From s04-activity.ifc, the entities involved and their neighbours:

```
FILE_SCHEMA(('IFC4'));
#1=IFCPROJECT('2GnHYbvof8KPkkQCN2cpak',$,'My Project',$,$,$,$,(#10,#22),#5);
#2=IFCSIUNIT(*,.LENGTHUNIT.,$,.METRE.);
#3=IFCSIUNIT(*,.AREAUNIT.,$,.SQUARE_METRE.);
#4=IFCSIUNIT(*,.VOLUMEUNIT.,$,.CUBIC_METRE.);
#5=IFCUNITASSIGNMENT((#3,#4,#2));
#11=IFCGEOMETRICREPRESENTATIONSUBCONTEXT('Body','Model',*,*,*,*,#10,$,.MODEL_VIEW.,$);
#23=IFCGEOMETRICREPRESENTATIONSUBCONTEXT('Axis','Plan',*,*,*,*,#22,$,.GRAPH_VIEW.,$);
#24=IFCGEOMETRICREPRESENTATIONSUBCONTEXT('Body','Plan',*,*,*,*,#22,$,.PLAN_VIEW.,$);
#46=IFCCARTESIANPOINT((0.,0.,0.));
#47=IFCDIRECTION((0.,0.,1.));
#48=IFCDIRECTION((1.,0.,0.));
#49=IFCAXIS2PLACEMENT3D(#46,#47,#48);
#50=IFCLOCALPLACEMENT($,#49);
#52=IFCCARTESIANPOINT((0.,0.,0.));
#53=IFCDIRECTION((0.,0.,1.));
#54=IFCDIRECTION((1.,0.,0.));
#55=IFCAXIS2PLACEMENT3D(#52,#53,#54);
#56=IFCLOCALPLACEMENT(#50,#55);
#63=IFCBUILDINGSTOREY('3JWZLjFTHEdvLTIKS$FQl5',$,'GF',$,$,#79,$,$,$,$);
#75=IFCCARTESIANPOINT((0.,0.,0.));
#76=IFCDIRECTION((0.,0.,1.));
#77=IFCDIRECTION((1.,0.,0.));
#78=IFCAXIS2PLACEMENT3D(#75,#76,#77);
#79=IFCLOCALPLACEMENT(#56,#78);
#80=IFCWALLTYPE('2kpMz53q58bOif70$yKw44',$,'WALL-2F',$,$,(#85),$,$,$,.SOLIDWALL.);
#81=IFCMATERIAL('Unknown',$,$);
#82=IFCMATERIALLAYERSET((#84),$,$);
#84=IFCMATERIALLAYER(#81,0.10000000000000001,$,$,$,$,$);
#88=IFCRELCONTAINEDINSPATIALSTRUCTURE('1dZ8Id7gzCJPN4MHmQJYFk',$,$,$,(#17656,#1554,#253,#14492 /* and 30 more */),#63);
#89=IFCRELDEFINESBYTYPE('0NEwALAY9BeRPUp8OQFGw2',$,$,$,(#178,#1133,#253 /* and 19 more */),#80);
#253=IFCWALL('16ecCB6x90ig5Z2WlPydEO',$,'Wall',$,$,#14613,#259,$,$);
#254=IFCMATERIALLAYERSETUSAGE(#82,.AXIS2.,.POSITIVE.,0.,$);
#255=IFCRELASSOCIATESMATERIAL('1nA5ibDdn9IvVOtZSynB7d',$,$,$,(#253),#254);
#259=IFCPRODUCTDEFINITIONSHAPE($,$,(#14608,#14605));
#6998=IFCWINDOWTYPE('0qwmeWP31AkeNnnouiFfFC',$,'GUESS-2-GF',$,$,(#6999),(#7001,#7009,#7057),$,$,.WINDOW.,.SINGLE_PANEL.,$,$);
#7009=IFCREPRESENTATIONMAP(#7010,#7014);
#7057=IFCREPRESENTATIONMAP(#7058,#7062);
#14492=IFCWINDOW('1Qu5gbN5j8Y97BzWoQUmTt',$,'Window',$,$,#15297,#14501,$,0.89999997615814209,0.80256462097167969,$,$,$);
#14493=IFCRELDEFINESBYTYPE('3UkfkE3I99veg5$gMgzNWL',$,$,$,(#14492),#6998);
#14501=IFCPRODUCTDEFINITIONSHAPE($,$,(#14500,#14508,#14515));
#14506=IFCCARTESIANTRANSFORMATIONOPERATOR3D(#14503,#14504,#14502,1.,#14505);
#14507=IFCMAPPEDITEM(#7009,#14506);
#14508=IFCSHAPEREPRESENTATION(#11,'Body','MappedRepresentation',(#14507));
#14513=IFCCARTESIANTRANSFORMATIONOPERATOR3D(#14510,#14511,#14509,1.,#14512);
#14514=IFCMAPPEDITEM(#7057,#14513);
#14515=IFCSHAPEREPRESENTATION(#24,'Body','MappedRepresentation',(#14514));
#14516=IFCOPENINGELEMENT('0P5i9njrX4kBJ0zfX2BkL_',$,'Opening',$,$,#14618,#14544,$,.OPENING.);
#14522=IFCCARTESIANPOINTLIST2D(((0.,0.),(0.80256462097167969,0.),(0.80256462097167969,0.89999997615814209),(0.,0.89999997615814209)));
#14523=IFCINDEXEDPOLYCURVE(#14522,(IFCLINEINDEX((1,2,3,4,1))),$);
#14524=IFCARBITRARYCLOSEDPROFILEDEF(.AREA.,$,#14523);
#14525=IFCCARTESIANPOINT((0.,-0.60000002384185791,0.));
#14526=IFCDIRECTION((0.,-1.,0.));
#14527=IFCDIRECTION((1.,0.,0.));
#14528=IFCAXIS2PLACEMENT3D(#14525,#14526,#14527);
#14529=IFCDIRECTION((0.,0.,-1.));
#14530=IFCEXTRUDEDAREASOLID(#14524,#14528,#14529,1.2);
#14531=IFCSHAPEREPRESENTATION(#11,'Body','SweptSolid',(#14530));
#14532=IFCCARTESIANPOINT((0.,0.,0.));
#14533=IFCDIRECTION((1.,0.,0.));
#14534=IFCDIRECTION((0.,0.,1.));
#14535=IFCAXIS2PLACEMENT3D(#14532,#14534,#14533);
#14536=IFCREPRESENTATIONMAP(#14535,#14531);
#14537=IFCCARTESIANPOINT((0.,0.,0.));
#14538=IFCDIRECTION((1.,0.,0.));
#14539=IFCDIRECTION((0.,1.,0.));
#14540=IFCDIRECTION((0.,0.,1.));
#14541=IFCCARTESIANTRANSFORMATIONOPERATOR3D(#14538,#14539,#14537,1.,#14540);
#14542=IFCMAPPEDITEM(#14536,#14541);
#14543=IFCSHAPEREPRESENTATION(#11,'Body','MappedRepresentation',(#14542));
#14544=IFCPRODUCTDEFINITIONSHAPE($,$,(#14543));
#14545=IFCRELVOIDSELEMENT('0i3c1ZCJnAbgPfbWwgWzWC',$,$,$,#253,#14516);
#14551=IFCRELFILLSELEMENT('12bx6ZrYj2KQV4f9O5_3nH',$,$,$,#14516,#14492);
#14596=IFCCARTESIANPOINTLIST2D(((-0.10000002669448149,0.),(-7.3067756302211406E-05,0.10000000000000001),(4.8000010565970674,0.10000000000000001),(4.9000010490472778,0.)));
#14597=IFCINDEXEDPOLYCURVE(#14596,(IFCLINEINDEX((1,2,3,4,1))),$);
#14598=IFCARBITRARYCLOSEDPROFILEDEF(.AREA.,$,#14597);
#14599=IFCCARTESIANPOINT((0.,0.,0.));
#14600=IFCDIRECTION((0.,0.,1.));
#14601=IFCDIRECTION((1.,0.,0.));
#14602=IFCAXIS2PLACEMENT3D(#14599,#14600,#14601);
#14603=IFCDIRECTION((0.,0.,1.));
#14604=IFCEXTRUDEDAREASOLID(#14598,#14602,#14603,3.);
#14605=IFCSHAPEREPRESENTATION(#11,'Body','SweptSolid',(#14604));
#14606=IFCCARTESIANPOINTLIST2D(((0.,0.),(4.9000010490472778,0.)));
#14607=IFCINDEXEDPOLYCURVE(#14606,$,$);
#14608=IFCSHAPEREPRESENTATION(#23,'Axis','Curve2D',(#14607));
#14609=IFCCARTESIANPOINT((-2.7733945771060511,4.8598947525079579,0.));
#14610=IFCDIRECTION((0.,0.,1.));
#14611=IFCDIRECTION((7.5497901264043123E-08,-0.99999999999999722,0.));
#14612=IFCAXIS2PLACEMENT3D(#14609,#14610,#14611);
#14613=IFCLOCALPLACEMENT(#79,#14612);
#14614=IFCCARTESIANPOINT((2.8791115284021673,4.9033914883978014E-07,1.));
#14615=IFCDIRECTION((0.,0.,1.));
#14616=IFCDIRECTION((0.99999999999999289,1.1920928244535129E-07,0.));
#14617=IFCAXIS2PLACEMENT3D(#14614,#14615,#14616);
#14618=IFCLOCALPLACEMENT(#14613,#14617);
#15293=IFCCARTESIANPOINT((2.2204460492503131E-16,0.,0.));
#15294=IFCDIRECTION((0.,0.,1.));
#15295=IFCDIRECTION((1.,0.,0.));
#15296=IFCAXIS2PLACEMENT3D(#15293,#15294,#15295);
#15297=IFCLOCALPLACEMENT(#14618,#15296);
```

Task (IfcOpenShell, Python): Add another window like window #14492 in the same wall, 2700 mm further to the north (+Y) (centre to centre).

```python
import ifcopenshell
import ifcopenshell.api.feature
import ifcopenshell.api.geometry
import ifcopenshell.api.root
import ifcopenshell.geom
import ifcopenshell.util.element
import ifcopenshell.util.placement
import ifcopenshell.util.shape
import ifcopenshell.util.unit

model = ifcopenshell.open("s04-activity.ifc")
unit_scale = ifcopenshell.util.unit.calculate_unit_scale(model)
settings = ifcopenshell.geom.settings()


def volume(element):
    """Net volume in cubic metres, openings subtracted."""
    shape = ifcopenshell.geom.create_shape(settings, element)
    return ifcopenshell.util.shape.get_volume(shape.geometry)


window = model.by_guid("1Qu5gbN5j8Y97BzWoQUmTt")
opening = window.FillsVoids[0].RelatingOpeningElement
wall = opening.VoidsElements[0].RelatingBuildingElement
before = volume(wall)
shift = ifcopenshell.util.placement.get_local_placement(wall.ObjectPlacement)[:3, 0] * -2.7 / unit_scale

# copy_class copies the void relationship, type, container and properties, but no geometry.
new_opening = ifcopenshell.api.root.copy_class(model, product=opening)
new_opening.Representation = ifcopenshell.util.element.copy_deep(
    model, opening.Representation, exclude=["IfcGeometricRepresentationContext", "IfcRepresentationMap"]
)
new_window = ifcopenshell.api.root.copy_class(model, product=window)
new_window.Representation = ifcopenshell.util.element.copy_deep(
    model, window.Representation, exclude=["IfcGeometricRepresentationContext", "IfcRepresentationMap"]
)
ifcopenshell.api.feature.add_filling(model, opening=new_opening, element=new_window)

for old, new in ((opening, new_opening), (window, new_window)):
    matrix = ifcopenshell.util.placement.get_local_placement(old.ObjectPlacement)
    matrix[:3, 3] += shift
    ifcopenshell.api.geometry.edit_object_placement(model, product=new, matrix=matrix, is_si=False)

after = volume(wall)

print(f"wall volume {before:.3f} -> {after:.3f} m3")

model.write("s04-activity_rev.ifc")
```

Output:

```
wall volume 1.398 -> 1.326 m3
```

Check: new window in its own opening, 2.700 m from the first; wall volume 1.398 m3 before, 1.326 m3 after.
